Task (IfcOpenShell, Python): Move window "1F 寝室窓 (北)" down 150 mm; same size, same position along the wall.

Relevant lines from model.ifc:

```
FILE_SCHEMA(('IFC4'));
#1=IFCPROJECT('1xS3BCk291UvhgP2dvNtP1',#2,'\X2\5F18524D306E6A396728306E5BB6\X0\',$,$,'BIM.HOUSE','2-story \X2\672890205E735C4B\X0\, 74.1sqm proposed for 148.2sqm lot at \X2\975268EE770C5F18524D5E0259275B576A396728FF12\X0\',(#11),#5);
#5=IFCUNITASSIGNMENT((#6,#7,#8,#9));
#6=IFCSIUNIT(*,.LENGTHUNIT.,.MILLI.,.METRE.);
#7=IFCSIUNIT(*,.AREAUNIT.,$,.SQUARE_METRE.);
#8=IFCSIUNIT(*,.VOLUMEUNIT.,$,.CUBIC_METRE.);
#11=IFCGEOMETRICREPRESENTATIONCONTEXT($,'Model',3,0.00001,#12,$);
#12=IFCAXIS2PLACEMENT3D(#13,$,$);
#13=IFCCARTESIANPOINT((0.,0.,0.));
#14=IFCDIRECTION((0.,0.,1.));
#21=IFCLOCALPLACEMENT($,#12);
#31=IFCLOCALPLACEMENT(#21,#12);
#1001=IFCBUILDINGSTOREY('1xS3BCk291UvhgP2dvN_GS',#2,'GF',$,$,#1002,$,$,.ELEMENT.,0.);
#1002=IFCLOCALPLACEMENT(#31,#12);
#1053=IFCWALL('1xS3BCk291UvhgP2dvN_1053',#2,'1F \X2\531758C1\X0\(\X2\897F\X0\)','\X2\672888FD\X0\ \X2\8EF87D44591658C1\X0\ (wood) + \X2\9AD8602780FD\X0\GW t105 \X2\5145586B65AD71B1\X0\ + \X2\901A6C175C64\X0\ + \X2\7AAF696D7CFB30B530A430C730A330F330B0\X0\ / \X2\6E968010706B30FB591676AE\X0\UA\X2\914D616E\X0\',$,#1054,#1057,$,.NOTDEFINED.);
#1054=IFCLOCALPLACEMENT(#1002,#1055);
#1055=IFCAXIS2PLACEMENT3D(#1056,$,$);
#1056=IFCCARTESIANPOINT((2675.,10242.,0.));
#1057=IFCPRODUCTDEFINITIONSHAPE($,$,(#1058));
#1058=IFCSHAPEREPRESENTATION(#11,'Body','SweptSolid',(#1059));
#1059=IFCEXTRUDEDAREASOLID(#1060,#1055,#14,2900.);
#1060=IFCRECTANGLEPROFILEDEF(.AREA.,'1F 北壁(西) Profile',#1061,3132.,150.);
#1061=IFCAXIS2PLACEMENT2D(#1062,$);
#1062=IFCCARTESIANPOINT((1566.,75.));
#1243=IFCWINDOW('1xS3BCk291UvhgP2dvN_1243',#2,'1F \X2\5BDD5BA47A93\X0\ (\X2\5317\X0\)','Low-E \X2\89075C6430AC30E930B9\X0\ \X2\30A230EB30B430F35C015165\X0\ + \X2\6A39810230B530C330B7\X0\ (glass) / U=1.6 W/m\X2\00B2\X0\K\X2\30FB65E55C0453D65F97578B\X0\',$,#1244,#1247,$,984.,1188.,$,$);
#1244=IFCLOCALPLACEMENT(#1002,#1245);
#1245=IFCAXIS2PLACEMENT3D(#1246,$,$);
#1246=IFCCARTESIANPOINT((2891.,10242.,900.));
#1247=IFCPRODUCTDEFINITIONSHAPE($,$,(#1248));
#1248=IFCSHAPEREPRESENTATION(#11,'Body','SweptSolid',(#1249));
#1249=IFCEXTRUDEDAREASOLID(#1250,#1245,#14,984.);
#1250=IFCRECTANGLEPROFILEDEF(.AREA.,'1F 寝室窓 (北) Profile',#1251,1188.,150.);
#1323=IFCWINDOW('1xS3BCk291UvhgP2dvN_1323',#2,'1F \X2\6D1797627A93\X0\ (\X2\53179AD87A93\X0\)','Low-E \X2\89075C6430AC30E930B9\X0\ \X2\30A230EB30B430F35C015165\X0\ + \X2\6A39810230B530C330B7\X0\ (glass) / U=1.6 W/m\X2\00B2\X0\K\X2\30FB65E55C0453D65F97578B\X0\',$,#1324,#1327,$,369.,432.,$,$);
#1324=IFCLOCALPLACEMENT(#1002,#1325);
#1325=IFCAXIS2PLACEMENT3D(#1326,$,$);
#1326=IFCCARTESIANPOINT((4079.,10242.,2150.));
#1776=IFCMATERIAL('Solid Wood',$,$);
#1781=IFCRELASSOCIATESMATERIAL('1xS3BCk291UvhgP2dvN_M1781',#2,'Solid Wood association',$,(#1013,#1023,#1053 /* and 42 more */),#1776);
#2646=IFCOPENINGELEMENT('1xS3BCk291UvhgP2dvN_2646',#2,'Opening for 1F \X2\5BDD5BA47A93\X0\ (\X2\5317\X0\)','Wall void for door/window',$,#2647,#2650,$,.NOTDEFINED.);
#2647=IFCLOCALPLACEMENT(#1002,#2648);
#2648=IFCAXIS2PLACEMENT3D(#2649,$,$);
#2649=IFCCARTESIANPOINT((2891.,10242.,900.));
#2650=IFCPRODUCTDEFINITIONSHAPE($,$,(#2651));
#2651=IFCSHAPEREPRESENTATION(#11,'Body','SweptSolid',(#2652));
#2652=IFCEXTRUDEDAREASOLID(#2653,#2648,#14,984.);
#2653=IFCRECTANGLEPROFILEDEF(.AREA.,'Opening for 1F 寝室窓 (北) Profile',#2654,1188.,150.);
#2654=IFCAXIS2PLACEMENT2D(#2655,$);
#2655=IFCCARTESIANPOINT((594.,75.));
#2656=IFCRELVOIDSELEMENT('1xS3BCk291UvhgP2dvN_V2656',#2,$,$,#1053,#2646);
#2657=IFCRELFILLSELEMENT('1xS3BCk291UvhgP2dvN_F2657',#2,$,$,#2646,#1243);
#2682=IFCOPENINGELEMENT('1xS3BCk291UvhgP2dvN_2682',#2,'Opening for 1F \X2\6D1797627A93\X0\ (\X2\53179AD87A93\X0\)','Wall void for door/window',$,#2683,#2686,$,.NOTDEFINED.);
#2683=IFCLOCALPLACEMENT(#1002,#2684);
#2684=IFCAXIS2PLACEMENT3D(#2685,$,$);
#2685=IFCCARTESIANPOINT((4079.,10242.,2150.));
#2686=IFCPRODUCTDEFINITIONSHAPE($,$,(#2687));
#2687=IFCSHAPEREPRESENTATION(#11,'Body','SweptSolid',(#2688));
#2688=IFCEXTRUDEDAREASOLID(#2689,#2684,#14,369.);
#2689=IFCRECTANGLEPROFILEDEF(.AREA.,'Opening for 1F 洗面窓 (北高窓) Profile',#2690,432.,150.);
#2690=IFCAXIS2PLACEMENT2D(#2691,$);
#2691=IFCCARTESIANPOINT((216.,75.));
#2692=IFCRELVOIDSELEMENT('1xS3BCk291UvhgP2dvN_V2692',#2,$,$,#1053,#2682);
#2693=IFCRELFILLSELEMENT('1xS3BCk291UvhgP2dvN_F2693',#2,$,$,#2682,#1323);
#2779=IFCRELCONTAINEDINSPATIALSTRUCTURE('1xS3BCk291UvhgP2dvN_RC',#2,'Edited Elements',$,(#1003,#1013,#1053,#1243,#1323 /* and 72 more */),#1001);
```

```python
import numpy as np
import ifcopenshell
import ifcopenshell.api.geometry
import ifcopenshell.util.placement
import ifcopenshell.util.unit

model = ifcopenshell.open("model.ifc")
unit_scale = ifcopenshell.util.unit.calculate_unit_scale(model)

window = model.by_id(1243)
opening = window.FillsVoids[0].RelatingOpeningElement
dz = -0.15 / unit_scale

shift = np.array([0.0, 0.0, dz])
# The window is not placed relative to its opening, so move both.
for product in (opening, window):
    matrix = ifcopenshell.util.placement.get_local_placement(product.ObjectPlacement)
    matrix[:3, 3] += shift
    ifcopenshell.api.geometry.edit_object_placement(model, product=product, matrix=matrix, is_si=False)

print(f"moved by {dz * unit_scale:+.3f} m")

model.write("model-out.ifc")
```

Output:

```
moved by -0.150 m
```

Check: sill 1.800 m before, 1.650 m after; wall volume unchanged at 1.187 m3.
